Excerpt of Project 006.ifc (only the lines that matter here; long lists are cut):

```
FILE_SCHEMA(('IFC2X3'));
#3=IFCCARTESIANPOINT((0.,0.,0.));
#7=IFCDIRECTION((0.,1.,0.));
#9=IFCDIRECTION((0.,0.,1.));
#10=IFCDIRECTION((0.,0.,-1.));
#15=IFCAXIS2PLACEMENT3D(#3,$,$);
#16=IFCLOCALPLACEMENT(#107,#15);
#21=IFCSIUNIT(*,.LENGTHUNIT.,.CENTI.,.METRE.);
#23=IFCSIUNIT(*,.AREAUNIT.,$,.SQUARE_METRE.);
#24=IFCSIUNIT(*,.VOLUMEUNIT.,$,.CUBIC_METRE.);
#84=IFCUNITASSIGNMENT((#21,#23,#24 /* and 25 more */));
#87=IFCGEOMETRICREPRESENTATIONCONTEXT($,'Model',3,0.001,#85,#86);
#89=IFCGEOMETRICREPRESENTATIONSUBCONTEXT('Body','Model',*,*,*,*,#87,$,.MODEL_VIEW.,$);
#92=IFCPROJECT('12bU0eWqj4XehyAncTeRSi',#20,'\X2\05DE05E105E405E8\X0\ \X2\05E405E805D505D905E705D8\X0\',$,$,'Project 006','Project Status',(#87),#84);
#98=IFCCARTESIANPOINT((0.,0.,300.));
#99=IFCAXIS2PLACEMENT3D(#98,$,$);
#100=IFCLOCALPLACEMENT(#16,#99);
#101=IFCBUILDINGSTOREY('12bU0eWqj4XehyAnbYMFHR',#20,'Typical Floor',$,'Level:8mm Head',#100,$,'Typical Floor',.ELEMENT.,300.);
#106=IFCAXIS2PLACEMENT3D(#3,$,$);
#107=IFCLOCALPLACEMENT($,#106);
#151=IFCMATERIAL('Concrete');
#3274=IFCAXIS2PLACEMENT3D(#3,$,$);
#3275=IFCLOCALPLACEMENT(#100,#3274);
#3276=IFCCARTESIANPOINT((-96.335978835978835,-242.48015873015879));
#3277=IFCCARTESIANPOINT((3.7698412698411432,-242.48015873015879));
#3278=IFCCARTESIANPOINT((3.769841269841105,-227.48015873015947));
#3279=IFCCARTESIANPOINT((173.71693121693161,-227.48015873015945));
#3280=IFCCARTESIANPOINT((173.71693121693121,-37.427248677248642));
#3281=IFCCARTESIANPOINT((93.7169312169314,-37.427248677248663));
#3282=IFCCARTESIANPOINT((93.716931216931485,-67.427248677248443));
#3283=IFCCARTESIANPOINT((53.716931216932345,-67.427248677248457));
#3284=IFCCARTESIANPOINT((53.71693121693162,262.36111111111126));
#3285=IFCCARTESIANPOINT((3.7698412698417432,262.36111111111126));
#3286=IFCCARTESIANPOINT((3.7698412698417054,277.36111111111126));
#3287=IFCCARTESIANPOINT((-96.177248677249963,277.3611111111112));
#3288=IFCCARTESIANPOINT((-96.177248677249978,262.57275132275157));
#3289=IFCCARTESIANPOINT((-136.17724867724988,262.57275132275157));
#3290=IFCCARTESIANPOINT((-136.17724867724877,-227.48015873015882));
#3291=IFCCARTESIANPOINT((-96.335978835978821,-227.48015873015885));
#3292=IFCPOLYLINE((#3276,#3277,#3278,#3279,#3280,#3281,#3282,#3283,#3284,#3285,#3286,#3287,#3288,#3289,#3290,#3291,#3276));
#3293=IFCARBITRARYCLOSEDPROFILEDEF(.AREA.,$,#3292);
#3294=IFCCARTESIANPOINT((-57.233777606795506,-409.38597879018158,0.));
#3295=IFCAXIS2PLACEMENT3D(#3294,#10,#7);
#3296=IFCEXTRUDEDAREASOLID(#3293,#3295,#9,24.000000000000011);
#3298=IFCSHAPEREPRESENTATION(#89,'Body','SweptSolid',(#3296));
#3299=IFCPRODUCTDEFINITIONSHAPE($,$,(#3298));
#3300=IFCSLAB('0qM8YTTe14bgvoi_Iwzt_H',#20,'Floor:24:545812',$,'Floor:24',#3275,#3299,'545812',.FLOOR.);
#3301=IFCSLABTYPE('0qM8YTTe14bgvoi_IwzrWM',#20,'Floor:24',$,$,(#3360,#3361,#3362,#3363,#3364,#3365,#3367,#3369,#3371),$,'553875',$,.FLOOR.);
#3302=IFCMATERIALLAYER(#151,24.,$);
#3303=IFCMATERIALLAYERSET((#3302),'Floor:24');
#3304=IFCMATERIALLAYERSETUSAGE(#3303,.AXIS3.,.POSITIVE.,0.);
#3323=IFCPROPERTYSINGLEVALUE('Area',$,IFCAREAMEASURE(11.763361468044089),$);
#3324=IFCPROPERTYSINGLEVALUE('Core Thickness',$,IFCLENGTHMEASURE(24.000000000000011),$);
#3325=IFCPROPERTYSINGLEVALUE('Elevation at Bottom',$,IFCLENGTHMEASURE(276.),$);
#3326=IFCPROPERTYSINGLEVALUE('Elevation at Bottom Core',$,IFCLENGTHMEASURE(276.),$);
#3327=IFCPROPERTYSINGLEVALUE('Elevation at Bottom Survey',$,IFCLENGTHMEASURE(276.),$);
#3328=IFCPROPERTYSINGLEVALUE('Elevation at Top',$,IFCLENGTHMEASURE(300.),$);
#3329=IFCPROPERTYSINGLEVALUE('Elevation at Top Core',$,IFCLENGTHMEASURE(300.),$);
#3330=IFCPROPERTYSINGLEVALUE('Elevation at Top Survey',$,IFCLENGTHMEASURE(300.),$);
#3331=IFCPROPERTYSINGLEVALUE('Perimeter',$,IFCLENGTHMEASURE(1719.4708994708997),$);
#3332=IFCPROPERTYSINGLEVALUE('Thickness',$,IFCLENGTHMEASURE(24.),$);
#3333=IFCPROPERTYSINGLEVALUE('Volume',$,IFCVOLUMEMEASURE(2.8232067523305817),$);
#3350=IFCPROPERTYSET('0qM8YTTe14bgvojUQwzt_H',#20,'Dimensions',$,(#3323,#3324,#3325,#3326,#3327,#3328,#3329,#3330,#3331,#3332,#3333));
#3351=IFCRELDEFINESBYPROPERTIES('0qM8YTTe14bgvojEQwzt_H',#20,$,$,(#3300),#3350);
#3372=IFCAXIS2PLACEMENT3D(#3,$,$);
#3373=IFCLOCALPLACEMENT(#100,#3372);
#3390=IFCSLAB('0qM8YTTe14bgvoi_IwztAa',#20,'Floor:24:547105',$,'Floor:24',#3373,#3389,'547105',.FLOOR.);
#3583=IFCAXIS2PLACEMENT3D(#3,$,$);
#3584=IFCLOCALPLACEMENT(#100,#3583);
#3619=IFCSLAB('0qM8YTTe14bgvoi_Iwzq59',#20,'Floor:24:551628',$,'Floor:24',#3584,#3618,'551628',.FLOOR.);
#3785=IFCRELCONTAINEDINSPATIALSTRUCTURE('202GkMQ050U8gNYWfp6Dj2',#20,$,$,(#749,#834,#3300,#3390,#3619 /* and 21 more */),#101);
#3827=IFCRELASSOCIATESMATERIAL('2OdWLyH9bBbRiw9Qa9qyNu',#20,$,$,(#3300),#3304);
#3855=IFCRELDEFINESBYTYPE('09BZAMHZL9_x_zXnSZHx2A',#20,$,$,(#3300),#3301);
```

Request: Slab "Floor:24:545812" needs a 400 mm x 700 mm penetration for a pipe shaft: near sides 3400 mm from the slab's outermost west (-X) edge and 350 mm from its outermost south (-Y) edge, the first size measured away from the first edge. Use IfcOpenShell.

```python
import numpy as np
import ifcopenshell
import ifcopenshell.api.feature
import ifcopenshell.api.geometry
import ifcopenshell.api.pset
import ifcopenshell.api.root
import ifcopenshell.geom
import ifcopenshell.util.element
import ifcopenshell.util.placement
import ifcopenshell.util.representation
import ifcopenshell.util.shape
import ifcopenshell.util.unit

model = ifcopenshell.open("Project 006.ifc")
unit_scale = ifcopenshell.util.unit.calculate_unit_scale(model)
area_scale = ifcopenshell.util.unit.calculate_unit_scale(model, "AREAUNIT")
volume_scale = ifcopenshell.util.unit.calculate_unit_scale(model, "VOLUMEUNIT")
settings = ifcopenshell.geom.settings()


def volume(element):
    """Net volume in cubic metres, openings subtracted."""
    shape = ifcopenshell.geom.create_shape(settings, element)
    return ifcopenshell.util.shape.get_volume(shape.geometry)


slab = model.by_guid("0qM8YTTe14bgvoi_Iwzt_H")
before = volume(slab)

# Extent in the slab's own axes, in metres. The edges named are its -X and -Y sides.
slab_shape = ifcopenshell.geom.create_shape(settings, slab)
vertices = ifcopenshell.util.shape.get_vertices(slab_shape.geometry)
x_min, y_min, bottom = vertices.min(axis=0)
top = vertices[:, 2].max()

opening = ifcopenshell.api.root.create_entity(model, ifc_class="IfcOpeningElement", name="Pipe shaft opening")
context = ifcopenshell.util.representation.get_context(model, "Model", "Body", "MODEL_VIEW")
width, depth = 0.4, 0.7
outline = [(0.0, 0.0), (width, 0.0), (width, depth), (0.0, depth), (0.0, 0.0)]
# Overshoot both faces by 50 mm so the cut is clean.
shape = ifcopenshell.api.geometry.add_slab_representation(
    model, context=context, depth=top - bottom + 0.1, polyline=outline
)
ifcopenshell.api.geometry.assign_representation(model, product=opening, representation=shape)

matrix = ifcopenshell.util.placement.get_local_placement(slab.ObjectPlacement)
matrix[:, 3] = matrix @ np.append(np.array([x_min + 3.4, y_min + 0.35, bottom - 0.05]) / unit_scale, 1.0)
ifcopenshell.api.geometry.edit_object_placement(model, product=opening, matrix=matrix, is_si=False)
ifcopenshell.api.feature.add_feature(model, feature=opening, element=slab)

after = volume(slab)

# Update the slab's stored quantities.
pset = model.by_id(ifcopenshell.util.element.get_pset(slab, "Dimensions", should_inherit=False)["id"])
ifcopenshell.api.pset.edit_pset(model, pset=pset, properties={
    "Area": model.create_entity("IfcAreaMeasure", after / (top - bottom) / area_scale),
    "Volume": model.create_entity("IfcVolumeMeasure", after / volume_scale),
})

print(f"slab volume {before:.3f} -> {after:.3f} m3")

model.write("Project 006_updated.ifc")
```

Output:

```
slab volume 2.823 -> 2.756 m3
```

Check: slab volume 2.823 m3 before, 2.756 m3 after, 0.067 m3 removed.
